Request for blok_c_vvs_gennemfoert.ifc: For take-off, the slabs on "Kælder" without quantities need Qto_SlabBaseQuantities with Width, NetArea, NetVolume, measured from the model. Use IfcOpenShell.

First a look at what the model holds.

```python
import ifcopenshell
import ifcopenshell.util.element
import ifcopenshell.util.unit

model = ifcopenshell.open("blok_c_vvs_gennemfoert.ifc")
print(model.schema)
for unit_type in ("LENGTHUNIT", "AREAUNIT", "VOLUMEUNIT"):
    print(unit_type, ifcopenshell.util.unit.calculate_unit_scale(model, unit_type))
storey = next(s for s in model.by_type("IfcBuildingStorey") if s.Name == "Kælder")
slabs = [e for e in ifcopenshell.util.element.get_decomposition(storey) if e.is_a("IfcSlab")]
for e in sorted(slabs, key=lambda e: e.id()):
    print(e.id(), e.is_a(), e.Name, list(ifcopenshell.util.element.get_psets(e, qtos_only=True)), sep=" | ")
```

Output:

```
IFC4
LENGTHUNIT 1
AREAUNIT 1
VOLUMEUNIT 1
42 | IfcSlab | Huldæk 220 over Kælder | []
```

```python
import ifcopenshell
import ifcopenshell.api.pset
import ifcopenshell.geom
import ifcopenshell.util.element
import ifcopenshell.util.shape
import ifcopenshell.util.unit

model = ifcopenshell.open("blok_c_vvs_gennemfoert.ifc")
unit_scale = ifcopenshell.util.unit.calculate_unit_scale(model)
area_scale = ifcopenshell.util.unit.calculate_unit_scale(model, "AREAUNIT")
volume_scale = ifcopenshell.util.unit.calculate_unit_scale(model, "VOLUMEUNIT")
settings = ifcopenshell.geom.settings()

storey = next(s for s in model.by_type("IfcBuildingStorey") if s.Name == "Kælder")
slabs = [e for e in ifcopenshell.util.element.get_decomposition(storey) if e.is_a("IfcSlab")]

for e in sorted(slabs, key=lambda e: e.id()):
    if ifcopenshell.util.element.get_psets(e, qtos_only=True, should_inherit=False):
        continue
    # Geometry comes back in metres, in the element's own axes.
    shape = ifcopenshell.geom.create_shape(settings, e)
    values = {
        "Width": ifcopenshell.util.shape.get_z(shape.geometry) / unit_scale,
        "NetArea": ifcopenshell.util.shape.get_footprint_area(shape.geometry) / area_scale,
        "NetVolume": ifcopenshell.util.shape.get_volume(shape.geometry) / volume_scale,
    }
    qto = ifcopenshell.api.pset.add_qto(model, product=e, name="Qto_SlabBaseQuantities")
    ifcopenshell.api.pset.edit_qto(model, qto=qto, properties=values)
    print(e.id(), {k: round(v, 3) for k, v in values.items()})

model.write("blok_c_vvs_gennemfoert_edited.ifc")
```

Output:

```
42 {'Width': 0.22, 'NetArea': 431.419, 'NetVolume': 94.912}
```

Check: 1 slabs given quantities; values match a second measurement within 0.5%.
